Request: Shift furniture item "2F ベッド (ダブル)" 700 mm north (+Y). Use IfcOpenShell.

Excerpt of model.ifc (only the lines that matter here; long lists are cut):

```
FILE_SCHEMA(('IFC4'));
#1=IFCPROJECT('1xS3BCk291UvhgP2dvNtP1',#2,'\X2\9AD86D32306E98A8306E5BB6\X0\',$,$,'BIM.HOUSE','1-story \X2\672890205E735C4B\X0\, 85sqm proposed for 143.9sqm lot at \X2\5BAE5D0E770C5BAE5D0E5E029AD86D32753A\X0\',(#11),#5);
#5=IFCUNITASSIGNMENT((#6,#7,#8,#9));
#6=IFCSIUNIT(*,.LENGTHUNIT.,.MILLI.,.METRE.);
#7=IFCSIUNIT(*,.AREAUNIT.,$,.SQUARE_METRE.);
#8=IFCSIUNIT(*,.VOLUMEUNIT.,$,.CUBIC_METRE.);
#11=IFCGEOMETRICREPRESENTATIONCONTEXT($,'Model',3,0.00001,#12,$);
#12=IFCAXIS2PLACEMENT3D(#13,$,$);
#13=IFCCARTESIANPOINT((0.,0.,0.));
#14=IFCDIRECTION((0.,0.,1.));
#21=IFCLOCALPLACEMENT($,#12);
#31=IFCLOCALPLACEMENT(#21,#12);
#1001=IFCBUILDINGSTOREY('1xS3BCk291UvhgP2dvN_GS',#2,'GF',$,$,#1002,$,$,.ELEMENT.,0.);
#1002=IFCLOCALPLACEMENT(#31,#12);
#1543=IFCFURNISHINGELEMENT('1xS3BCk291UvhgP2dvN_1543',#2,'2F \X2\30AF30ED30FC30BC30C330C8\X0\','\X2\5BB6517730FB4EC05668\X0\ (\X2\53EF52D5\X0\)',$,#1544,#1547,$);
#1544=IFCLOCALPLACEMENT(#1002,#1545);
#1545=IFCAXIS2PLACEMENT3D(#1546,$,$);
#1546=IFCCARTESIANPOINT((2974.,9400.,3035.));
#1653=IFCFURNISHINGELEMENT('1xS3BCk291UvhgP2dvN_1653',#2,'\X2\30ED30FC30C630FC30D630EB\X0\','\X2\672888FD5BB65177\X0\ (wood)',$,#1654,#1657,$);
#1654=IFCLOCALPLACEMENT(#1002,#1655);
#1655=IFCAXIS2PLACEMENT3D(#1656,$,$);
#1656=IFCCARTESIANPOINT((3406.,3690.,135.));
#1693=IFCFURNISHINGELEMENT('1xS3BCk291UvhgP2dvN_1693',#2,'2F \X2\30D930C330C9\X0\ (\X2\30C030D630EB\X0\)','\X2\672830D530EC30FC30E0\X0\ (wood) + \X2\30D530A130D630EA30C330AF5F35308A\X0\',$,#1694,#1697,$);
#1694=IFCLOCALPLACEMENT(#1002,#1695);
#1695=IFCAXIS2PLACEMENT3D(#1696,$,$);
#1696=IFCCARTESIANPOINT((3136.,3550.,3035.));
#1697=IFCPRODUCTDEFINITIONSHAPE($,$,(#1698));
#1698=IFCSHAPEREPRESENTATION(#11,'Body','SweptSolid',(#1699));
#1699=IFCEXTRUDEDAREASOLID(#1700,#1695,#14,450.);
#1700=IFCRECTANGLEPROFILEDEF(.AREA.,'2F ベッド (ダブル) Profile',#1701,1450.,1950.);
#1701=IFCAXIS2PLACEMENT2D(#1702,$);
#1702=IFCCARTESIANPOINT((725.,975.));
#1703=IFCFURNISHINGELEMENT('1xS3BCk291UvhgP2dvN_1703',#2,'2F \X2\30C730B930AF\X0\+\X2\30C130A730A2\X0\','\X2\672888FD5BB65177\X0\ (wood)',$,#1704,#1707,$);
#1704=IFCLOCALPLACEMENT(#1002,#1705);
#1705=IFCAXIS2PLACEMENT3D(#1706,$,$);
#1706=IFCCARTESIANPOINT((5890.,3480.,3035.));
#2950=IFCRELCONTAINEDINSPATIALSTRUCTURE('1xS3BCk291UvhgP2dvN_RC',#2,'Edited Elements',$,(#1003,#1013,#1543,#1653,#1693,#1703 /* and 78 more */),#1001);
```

```python
import ifcopenshell
import ifcopenshell.api.geometry
import ifcopenshell.util.placement
import ifcopenshell.util.unit

model = ifcopenshell.open("model.ifc")
unit_scale = ifcopenshell.util.unit.calculate_unit_scale(model)

item = model.by_id(1693)
matrix = ifcopenshell.util.placement.get_local_placement(item.ObjectPlacement)
matrix[1, 3] += 0.7 / unit_scale
ifcopenshell.api.geometry.edit_object_placement(model, product=item, matrix=matrix, is_si=False)

print(ifcopenshell.util.placement.get_local_placement(item.ObjectPlacement).round(3) + 0.0)

model.write("model_v2.ifc")
```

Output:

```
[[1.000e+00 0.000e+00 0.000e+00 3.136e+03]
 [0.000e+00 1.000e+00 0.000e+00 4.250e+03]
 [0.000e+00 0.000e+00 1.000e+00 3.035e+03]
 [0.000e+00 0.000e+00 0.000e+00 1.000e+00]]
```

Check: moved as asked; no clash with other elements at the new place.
